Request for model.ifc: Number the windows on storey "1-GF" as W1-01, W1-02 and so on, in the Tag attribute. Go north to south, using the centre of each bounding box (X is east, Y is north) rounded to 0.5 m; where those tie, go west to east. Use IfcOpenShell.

First a look at what the model holds.

```python
import ifcopenshell
import ifcopenshell.util.element
import ifcopenshell.util.placement

model = ifcopenshell.open("model.ifc")
print(model.schema)
storey = next(s for s in model.by_type("IfcBuildingStorey") if s.Name == "1-GF")
windows = [e for e in ifcopenshell.util.element.get_decomposition(storey) if e.is_a("IfcWindow")]
for e in sorted(windows, key=lambda e: e.id()):
    origin = ifcopenshell.util.placement.get_local_placement(e.ObjectPlacement)[:3, 3]
    print(e.id(), e.Tag, e.Name, origin.round(2) + 0.0, sep=" | ")
```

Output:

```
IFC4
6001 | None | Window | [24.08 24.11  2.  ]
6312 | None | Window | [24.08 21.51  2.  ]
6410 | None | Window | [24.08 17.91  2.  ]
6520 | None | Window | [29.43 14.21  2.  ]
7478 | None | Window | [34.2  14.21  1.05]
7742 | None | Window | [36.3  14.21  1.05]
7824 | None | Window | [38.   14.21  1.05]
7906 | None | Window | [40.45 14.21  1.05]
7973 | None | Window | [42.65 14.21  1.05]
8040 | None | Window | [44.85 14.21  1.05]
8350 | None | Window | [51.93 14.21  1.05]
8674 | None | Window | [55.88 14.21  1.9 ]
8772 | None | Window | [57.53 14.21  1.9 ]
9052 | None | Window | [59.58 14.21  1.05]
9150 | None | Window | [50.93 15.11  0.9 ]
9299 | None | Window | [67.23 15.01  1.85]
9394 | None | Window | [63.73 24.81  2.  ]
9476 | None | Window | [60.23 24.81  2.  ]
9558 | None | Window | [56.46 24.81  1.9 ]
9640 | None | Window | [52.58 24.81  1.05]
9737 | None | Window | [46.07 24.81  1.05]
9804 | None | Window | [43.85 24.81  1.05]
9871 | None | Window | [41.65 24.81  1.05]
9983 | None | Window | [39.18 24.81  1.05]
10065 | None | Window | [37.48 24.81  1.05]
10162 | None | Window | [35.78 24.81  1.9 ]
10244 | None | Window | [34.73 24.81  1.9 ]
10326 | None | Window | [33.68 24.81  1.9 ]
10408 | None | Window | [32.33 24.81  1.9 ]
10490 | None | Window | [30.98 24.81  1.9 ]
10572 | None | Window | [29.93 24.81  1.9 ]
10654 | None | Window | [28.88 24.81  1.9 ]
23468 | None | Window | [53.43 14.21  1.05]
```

```python
import ifcopenshell
import ifcopenshell.geom
import ifcopenshell.util.element
import ifcopenshell.util.shape

model = ifcopenshell.open("model.ifc")
settings = ifcopenshell.geom.settings()
settings.set("use-world-coords", True)


def centre(element):
    shape = ifcopenshell.geom.create_shape(settings, element)
    return ifcopenshell.util.shape.get_bbox_centroid(shape.geometry)


storey = next(s for s in model.by_type("IfcBuildingStorey") if s.Name == "1-GF")
windows = [e for e in ifcopenshell.util.element.get_decomposition(storey) if e.is_a("IfcWindow")]

# Insertion points can sit at a corner or the storey origin, so sort by the geometry (in metres).
centres = {e: centre(e) for e in windows}
windows.sort(key=lambda e: (-round(centres[e][1] / 0.5), centres[e][0]))

for i, e in enumerate(windows, start=1):
    number = f"W1-{i:02d}"
    e.Tag = number
    print(e.id(), number)

model.write("model_updated.ifc")
```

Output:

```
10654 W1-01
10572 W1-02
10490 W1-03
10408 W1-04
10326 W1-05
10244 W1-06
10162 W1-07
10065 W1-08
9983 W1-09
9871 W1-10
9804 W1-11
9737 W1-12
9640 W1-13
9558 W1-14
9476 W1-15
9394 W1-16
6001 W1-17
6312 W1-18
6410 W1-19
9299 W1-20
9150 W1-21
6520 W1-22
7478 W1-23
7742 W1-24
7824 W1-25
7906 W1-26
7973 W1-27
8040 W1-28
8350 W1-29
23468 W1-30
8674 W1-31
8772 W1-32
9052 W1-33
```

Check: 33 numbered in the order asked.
